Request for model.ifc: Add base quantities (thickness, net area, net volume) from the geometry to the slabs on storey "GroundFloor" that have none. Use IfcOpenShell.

First a look at what the model holds.

```python
import ifcopenshell
import ifcopenshell.util.element
import ifcopenshell.util.unit

model = ifcopenshell.open("model.ifc")
print(model.schema)
for unit_type in ("LENGTHUNIT", "AREAUNIT", "VOLUMEUNIT"):
    print(unit_type, ifcopenshell.util.unit.calculate_unit_scale(model, unit_type))
storey = next(s for s in model.by_type("IfcBuildingStorey") if s.Name == "GroundFloor")
slabs = [e for e in ifcopenshell.util.element.get_decomposition(storey) if e.is_a("IfcSlab")]
for e in sorted(slabs, key=lambda e: e.id()):
    print(e.id(), e.is_a(), e.Name, list(ifcopenshell.util.element.get_psets(e, qtos_only=True)), sep=" | ")
```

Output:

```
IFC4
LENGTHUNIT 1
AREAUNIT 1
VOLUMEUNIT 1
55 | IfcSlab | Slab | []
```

```python
import ifcopenshell
import ifcopenshell.api.pset
import ifcopenshell.geom
import ifcopenshell.util.element
import ifcopenshell.util.shape
import ifcopenshell.util.unit

model = ifcopenshell.open("model.ifc")
unit_scale = ifcopenshell.util.unit.calculate_unit_scale(model)
area_scale = ifcopenshell.util.unit.calculate_unit_scale(model, "AREAUNIT")
volume_scale = ifcopenshell.util.unit.calculate_unit_scale(model, "VOLUMEUNIT")
settings = ifcopenshell.geom.settings()

storey = next(s for s in model.by_type("IfcBuildingStorey") if s.Name == "GroundFloor")
slabs = [e for e in ifcopenshell.util.element.get_decomposition(storey) if e.is_a("IfcSlab")]

for e in sorted(slabs, key=lambda e: e.id()):
    if ifcopenshell.util.element.get_psets(e, qtos_only=True, should_inherit=False):
        continue
    # Geometry comes back in metres, in the element's own axes.
    shape = ifcopenshell.geom.create_shape(settings, e)
    values = {
        "Width": ifcopenshell.util.shape.get_z(shape.geometry) / unit_scale,
        "NetArea": ifcopenshell.util.shape.get_footprint_area(shape.geometry) / area_scale,
        "NetVolume": ifcopenshell.util.shape.get_volume(shape.geometry) / volume_scale,
    }
    qto = ifcopenshell.api.pset.add_qto(model, product=e, name="Qto_SlabBaseQuantities")
    ifcopenshell.api.pset.edit_qto(model, qto=qto, properties=values)
    print(e.id(), {k: round(v, 3) for k, v in values.items()})

model.write("model_v2.ifc")
```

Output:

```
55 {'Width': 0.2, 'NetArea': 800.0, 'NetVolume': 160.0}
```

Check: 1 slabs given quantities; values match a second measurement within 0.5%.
